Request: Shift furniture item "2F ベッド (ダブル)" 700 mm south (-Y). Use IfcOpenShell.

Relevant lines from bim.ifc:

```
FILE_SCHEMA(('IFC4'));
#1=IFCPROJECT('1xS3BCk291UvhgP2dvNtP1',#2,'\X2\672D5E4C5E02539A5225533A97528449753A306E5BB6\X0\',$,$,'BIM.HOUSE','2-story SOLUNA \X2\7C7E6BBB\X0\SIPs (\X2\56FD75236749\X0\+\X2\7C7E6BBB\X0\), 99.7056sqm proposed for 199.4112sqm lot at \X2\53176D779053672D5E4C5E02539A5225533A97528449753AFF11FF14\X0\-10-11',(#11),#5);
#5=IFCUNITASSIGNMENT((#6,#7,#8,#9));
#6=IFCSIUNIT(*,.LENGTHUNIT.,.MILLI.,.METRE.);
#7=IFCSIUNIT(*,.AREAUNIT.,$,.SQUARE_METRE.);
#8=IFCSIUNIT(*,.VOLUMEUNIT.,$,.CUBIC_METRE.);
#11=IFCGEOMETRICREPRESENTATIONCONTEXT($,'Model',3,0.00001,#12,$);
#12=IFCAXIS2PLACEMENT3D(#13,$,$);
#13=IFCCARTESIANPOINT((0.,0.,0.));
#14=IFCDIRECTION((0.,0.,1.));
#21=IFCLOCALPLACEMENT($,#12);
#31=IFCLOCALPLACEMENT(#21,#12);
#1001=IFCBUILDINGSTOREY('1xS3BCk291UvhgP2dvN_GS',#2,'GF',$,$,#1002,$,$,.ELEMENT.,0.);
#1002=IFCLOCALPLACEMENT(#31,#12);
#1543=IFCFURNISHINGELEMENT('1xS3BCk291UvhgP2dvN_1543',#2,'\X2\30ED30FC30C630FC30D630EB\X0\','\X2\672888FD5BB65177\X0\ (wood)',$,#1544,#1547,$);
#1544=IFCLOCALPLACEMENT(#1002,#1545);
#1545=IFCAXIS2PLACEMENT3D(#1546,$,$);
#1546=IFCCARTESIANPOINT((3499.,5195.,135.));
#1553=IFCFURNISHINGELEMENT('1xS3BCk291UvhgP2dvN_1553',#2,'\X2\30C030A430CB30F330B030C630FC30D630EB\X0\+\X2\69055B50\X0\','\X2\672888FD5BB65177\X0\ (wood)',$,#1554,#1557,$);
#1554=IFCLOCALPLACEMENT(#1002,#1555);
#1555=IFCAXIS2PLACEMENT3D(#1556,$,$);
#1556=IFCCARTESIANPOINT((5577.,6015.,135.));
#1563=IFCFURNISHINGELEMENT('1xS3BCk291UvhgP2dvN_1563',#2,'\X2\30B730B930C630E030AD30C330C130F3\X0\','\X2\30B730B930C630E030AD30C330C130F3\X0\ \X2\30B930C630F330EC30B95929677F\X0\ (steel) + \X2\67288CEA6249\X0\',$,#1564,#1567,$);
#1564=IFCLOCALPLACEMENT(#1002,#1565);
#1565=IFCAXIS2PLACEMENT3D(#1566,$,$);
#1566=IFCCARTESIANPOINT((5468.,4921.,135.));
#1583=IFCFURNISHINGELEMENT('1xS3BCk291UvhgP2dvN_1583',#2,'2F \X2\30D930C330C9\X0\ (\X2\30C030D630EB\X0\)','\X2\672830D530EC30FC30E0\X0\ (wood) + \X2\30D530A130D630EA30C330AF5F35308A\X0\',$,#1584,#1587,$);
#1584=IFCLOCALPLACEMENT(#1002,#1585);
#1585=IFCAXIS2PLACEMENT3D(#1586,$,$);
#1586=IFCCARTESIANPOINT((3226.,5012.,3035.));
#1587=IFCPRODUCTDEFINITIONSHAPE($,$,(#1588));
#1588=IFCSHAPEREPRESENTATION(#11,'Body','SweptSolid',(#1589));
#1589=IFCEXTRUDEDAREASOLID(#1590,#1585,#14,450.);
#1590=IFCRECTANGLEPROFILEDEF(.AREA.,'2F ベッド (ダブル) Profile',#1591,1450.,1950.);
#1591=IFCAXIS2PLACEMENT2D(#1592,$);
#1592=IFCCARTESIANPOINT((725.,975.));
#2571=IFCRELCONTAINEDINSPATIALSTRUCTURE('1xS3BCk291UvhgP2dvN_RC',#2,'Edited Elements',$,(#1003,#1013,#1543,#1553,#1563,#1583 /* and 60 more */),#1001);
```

```python
import ifcopenshell
import ifcopenshell.api.geometry
import ifcopenshell.util.placement
import ifcopenshell.util.unit

model = ifcopenshell.open("bim.ifc")
unit_scale = ifcopenshell.util.unit.calculate_unit_scale(model)

item = model.by_guid("1xS3BCk291UvhgP2dvN_1583")
matrix = ifcopenshell.util.placement.get_local_placement(item.ObjectPlacement)
matrix[1, 3] -= 0.7 / unit_scale
ifcopenshell.api.geometry.edit_object_placement(model, product=item, matrix=matrix, is_si=False)

print(ifcopenshell.util.placement.get_local_placement(item.ObjectPlacement).round(3) + 0.0)

model.write("bim_edited.ifc")
```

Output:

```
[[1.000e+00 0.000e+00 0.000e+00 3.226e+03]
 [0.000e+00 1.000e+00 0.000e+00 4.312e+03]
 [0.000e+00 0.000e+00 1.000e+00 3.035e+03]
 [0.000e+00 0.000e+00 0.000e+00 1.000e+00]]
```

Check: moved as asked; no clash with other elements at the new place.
